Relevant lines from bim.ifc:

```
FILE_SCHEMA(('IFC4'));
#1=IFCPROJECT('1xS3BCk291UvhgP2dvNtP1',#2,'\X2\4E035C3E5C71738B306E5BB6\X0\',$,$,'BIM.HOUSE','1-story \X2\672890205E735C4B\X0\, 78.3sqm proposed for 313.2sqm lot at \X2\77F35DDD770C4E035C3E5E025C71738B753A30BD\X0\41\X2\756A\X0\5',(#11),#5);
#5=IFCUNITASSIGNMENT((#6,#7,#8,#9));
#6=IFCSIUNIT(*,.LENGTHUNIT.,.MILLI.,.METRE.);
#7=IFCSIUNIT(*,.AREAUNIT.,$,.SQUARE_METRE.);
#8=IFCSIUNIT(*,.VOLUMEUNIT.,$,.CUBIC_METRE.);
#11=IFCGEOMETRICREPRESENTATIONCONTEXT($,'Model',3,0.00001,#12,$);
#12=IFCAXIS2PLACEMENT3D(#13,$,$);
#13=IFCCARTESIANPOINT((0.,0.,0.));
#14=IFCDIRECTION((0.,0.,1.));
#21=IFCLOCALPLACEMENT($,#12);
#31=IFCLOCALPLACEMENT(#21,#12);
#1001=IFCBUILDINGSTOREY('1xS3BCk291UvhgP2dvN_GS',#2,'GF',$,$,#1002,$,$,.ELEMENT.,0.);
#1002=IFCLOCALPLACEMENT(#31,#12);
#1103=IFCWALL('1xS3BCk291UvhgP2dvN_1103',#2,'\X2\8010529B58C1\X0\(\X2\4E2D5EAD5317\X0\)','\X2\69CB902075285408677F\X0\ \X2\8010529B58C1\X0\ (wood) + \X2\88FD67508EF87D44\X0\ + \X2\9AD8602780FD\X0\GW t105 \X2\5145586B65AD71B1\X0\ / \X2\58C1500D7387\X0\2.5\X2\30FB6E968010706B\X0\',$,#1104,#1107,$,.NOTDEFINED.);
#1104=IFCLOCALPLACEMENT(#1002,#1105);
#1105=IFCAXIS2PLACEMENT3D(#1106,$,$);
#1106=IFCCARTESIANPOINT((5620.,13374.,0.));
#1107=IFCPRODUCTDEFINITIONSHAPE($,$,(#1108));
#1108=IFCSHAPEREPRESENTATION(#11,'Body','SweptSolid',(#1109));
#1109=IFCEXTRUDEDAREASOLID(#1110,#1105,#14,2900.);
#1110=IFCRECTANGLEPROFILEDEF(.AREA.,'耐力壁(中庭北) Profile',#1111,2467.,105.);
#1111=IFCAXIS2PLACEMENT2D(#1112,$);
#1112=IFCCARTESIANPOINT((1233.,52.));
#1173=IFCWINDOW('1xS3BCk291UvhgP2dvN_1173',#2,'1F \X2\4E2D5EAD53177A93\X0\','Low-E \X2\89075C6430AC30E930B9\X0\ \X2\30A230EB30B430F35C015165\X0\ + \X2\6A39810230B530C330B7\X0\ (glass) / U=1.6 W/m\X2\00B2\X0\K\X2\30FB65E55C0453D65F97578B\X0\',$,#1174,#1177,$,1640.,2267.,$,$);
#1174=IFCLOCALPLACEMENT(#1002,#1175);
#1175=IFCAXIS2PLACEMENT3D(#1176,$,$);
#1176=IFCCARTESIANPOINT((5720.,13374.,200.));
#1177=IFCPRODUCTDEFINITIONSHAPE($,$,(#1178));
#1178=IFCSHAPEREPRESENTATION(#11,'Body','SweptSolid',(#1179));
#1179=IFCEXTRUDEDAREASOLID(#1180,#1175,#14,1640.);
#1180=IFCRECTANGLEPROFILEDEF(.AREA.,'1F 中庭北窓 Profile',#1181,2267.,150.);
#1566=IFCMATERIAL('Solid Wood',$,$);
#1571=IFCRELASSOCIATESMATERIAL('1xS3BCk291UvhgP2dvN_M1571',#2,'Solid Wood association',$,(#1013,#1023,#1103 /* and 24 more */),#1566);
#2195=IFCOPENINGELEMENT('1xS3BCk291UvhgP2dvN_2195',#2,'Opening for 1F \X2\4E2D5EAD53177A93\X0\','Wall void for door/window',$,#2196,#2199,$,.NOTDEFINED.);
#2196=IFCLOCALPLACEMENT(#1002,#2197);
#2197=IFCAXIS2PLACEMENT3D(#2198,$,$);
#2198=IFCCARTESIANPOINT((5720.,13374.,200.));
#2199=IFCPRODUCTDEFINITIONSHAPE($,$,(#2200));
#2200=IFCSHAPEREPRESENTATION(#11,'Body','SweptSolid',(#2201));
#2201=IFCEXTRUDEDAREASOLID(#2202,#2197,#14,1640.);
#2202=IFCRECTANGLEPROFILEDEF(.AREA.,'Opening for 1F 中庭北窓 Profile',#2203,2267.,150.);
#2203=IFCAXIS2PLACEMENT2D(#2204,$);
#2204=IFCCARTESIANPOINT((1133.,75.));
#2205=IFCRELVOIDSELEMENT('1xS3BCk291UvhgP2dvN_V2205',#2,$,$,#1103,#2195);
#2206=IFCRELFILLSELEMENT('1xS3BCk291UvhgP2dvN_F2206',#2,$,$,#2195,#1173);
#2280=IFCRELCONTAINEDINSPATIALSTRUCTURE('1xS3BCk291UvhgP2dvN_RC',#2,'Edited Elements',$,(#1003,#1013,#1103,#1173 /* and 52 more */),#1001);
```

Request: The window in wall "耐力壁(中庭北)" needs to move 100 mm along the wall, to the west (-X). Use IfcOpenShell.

```python
import ifcopenshell
import ifcopenshell.api.geometry
import ifcopenshell.util.placement

model = ifcopenshell.open("bim.ifc")

window = model.by_guid("1xS3BCk291UvhgP2dvN_1173")
opening = window.FillsVoids[0].RelatingOpeningElement
wall = opening.VoidsElements[0].RelatingBuildingElement

wall_matrix = ifcopenshell.util.placement.get_local_placement(wall.ObjectPlacement)
shift = wall_matrix[:3, 0] * -100.0
before = ifcopenshell.util.placement.get_local_placement(window.ObjectPlacement)[:3, 3].copy()

# The window is not placed relative to its opening, so move both.
for product in (opening, window):
    matrix = ifcopenshell.util.placement.get_local_placement(product.ObjectPlacement)
    matrix[:3, 3] += shift
    ifcopenshell.api.geometry.edit_object_placement(model, product=product, matrix=matrix, is_si=False)

after = ifcopenshell.util.placement.get_local_placement(window.ObjectPlacement)[:3, 3]
print("window moved by", (after - before).round(3) + 0.0)

model.write("bim_updated.ifc")
```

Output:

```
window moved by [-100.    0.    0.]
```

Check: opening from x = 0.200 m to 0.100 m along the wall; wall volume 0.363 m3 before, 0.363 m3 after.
